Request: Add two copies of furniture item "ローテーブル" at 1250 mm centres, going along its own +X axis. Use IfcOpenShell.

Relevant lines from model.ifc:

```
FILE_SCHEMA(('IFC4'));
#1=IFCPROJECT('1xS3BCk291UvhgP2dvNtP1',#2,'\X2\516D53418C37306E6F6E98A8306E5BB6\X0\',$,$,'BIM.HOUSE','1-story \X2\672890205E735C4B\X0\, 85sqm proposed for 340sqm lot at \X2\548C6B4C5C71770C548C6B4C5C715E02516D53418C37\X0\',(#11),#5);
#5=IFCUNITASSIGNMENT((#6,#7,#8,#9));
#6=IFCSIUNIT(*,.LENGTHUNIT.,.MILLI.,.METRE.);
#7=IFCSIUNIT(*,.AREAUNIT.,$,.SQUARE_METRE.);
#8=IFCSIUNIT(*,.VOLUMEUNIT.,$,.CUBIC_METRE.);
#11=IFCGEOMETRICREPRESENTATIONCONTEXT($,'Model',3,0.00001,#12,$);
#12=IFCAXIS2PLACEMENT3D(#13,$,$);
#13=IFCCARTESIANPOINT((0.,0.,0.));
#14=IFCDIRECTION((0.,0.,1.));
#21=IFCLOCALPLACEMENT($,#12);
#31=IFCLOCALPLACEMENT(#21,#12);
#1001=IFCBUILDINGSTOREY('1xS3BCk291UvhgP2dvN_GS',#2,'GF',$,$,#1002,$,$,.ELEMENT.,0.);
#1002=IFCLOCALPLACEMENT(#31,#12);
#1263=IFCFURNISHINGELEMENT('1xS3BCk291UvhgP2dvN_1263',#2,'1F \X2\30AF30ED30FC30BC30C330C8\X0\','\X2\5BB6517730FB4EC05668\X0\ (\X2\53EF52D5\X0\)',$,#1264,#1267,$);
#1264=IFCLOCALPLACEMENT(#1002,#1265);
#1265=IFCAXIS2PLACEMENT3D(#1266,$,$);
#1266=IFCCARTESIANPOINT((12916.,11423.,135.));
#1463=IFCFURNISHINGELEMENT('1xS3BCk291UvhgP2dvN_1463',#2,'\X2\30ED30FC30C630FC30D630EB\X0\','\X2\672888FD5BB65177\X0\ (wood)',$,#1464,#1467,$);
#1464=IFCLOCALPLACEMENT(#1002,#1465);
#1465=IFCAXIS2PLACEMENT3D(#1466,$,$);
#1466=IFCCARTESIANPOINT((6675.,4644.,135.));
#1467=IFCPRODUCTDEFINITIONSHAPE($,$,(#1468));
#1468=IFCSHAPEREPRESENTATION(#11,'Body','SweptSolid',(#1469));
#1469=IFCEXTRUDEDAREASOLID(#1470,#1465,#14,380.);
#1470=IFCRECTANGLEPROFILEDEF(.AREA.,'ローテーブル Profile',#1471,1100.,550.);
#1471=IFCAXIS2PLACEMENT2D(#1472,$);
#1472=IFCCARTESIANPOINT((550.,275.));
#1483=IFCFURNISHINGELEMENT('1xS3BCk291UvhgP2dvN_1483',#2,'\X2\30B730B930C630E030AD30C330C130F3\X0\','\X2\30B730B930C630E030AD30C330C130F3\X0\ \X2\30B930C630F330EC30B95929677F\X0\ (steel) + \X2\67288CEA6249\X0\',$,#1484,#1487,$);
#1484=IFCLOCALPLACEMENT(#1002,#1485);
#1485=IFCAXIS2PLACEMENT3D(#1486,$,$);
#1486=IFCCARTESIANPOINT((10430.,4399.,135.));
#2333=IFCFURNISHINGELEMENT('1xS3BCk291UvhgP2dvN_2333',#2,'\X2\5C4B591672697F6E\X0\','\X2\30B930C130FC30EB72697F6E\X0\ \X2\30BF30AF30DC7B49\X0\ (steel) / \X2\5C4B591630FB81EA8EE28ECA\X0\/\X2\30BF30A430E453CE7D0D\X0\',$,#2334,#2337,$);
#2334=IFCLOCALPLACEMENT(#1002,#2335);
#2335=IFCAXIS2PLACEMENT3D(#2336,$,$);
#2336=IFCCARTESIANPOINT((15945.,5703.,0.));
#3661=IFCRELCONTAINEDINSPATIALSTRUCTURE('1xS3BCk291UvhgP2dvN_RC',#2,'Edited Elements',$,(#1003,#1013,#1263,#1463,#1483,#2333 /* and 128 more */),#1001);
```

```python
import ifcopenshell
import ifcopenshell.api.geometry
import ifcopenshell.api.root
import ifcopenshell.util.element
import ifcopenshell.util.placement
import ifcopenshell.util.unit

model = ifcopenshell.open("model.ifc")
unit_scale = ifcopenshell.util.unit.calculate_unit_scale(model)


def reuse_history(source, copy):
    """copy_class also copies each property set's owner history, people and application; keep the originals."""
    for rel in copy.IsDefinedBy:
        if rel.is_a("IfcRelDefinesByProperties") and (history := rel.RelatingPropertyDefinition.OwnerHistory):
            rel.RelatingPropertyDefinition.OwnerHistory = source.OwnerHistory
            ifcopenshell.util.element.remove_deep2(model, history)


source = model.by_id(1463)
base = ifcopenshell.util.placement.get_local_placement(source.ObjectPlacement)
step = base[:3, 0] * 1.25 / unit_scale

for i in range(1, 3):
    copy = ifcopenshell.api.root.copy_class(model, product=source)
    copy.Representation = ifcopenshell.util.element.copy_deep(
        model, source.Representation, exclude=["IfcGeometricRepresentationContext", "IfcRepresentationMap"]
    )
    reuse_history(source, copy)
    matrix = base.copy()
    matrix[:3, 3] += i * step
    print("added at", matrix[:3, 3].round(3) + 0.0)
    ifcopenshell.api.geometry.edit_object_placement(model, product=copy, matrix=matrix, is_si=False)

model.write("model_edited.ifc")
```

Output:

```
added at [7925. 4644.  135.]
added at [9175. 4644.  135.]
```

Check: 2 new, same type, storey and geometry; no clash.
